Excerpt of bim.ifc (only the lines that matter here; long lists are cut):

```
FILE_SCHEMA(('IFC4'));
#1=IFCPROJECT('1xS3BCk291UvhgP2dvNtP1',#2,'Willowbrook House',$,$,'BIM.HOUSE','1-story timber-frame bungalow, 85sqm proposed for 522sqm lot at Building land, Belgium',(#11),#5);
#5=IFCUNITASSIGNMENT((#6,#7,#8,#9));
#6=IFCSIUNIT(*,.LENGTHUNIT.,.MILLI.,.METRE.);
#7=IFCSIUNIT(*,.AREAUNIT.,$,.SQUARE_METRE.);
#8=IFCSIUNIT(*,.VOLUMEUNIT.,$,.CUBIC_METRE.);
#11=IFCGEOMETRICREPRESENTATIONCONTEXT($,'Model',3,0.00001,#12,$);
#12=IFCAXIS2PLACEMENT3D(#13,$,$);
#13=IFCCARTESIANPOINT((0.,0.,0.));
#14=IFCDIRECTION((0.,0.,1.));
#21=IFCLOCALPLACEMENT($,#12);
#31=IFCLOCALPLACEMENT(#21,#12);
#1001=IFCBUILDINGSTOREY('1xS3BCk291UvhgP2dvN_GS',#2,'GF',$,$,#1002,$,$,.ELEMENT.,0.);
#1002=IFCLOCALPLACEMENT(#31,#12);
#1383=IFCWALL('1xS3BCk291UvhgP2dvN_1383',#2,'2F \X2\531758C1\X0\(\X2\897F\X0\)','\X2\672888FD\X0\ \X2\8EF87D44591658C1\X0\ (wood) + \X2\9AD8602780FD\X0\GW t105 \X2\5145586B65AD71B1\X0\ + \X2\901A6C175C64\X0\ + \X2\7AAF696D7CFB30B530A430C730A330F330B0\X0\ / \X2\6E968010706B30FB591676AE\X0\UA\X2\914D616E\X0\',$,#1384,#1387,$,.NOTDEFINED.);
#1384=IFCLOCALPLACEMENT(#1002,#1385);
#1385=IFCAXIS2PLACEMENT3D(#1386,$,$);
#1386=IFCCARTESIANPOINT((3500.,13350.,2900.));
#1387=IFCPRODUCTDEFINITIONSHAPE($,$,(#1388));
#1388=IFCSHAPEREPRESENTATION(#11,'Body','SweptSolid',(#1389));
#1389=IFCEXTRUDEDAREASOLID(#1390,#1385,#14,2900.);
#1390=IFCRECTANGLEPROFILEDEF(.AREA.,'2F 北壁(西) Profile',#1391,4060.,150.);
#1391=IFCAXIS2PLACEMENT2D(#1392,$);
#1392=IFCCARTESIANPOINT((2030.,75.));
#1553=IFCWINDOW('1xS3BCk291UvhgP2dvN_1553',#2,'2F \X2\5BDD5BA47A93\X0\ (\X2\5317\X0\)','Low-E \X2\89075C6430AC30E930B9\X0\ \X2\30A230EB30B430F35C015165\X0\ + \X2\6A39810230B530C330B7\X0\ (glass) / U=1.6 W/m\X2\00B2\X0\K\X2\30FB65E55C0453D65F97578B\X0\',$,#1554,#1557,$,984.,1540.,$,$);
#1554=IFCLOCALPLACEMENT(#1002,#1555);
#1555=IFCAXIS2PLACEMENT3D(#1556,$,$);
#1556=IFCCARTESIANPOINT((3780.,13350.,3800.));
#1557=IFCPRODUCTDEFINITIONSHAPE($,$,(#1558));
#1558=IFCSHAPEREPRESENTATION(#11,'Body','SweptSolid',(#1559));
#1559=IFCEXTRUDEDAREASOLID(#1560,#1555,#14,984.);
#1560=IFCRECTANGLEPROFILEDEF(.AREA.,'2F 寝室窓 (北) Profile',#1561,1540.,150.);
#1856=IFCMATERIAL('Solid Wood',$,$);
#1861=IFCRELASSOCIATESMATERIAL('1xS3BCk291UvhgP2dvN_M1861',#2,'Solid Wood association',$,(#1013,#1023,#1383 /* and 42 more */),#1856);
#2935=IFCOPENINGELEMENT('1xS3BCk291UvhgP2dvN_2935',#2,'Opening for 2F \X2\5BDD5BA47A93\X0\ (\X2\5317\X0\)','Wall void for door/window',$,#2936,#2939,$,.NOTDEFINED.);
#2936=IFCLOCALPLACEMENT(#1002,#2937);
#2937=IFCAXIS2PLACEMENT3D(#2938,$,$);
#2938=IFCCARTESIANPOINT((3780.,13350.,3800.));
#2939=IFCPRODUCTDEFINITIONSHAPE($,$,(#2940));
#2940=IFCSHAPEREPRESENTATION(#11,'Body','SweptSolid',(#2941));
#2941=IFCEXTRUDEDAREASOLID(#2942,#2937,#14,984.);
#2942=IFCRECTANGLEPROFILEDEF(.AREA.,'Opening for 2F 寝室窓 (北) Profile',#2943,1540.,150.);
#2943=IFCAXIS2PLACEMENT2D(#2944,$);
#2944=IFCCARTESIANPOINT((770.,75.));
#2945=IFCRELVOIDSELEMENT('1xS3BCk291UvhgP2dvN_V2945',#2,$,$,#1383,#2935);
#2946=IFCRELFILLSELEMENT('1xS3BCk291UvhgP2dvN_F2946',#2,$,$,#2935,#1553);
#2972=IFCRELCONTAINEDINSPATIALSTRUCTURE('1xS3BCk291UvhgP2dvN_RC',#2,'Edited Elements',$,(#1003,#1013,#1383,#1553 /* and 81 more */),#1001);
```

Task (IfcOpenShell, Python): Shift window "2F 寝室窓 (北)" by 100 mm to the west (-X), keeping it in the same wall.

```python
import ifcopenshell
import ifcopenshell.api.geometry
import ifcopenshell.util.placement

model = ifcopenshell.open("bim.ifc")

window = model.by_id(1553)
opening = window.FillsVoids[0].RelatingOpeningElement
wall = opening.VoidsElements[0].RelatingBuildingElement

wall_matrix = ifcopenshell.util.placement.get_local_placement(wall.ObjectPlacement)
shift = wall_matrix[:3, 0] * -100.0
before = ifcopenshell.util.placement.get_local_placement(window.ObjectPlacement)[:3, 3].copy()

# The window is not placed relative to its opening, so move both.
for product in (opening, window):
    matrix = ifcopenshell.util.placement.get_local_placement(product.ObjectPlacement)
    matrix[:3, 3] += shift
    ifcopenshell.api.geometry.edit_object_placement(model, product=product, matrix=matrix, is_si=False)

after = ifcopenshell.util.placement.get_local_placement(window.ObjectPlacement)[:3, 3]
print("window moved by", (after - before).round(3) + 0.0)

model.write("bim_v2.ifc")
```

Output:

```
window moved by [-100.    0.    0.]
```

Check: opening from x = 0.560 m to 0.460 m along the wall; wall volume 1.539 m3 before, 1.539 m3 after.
